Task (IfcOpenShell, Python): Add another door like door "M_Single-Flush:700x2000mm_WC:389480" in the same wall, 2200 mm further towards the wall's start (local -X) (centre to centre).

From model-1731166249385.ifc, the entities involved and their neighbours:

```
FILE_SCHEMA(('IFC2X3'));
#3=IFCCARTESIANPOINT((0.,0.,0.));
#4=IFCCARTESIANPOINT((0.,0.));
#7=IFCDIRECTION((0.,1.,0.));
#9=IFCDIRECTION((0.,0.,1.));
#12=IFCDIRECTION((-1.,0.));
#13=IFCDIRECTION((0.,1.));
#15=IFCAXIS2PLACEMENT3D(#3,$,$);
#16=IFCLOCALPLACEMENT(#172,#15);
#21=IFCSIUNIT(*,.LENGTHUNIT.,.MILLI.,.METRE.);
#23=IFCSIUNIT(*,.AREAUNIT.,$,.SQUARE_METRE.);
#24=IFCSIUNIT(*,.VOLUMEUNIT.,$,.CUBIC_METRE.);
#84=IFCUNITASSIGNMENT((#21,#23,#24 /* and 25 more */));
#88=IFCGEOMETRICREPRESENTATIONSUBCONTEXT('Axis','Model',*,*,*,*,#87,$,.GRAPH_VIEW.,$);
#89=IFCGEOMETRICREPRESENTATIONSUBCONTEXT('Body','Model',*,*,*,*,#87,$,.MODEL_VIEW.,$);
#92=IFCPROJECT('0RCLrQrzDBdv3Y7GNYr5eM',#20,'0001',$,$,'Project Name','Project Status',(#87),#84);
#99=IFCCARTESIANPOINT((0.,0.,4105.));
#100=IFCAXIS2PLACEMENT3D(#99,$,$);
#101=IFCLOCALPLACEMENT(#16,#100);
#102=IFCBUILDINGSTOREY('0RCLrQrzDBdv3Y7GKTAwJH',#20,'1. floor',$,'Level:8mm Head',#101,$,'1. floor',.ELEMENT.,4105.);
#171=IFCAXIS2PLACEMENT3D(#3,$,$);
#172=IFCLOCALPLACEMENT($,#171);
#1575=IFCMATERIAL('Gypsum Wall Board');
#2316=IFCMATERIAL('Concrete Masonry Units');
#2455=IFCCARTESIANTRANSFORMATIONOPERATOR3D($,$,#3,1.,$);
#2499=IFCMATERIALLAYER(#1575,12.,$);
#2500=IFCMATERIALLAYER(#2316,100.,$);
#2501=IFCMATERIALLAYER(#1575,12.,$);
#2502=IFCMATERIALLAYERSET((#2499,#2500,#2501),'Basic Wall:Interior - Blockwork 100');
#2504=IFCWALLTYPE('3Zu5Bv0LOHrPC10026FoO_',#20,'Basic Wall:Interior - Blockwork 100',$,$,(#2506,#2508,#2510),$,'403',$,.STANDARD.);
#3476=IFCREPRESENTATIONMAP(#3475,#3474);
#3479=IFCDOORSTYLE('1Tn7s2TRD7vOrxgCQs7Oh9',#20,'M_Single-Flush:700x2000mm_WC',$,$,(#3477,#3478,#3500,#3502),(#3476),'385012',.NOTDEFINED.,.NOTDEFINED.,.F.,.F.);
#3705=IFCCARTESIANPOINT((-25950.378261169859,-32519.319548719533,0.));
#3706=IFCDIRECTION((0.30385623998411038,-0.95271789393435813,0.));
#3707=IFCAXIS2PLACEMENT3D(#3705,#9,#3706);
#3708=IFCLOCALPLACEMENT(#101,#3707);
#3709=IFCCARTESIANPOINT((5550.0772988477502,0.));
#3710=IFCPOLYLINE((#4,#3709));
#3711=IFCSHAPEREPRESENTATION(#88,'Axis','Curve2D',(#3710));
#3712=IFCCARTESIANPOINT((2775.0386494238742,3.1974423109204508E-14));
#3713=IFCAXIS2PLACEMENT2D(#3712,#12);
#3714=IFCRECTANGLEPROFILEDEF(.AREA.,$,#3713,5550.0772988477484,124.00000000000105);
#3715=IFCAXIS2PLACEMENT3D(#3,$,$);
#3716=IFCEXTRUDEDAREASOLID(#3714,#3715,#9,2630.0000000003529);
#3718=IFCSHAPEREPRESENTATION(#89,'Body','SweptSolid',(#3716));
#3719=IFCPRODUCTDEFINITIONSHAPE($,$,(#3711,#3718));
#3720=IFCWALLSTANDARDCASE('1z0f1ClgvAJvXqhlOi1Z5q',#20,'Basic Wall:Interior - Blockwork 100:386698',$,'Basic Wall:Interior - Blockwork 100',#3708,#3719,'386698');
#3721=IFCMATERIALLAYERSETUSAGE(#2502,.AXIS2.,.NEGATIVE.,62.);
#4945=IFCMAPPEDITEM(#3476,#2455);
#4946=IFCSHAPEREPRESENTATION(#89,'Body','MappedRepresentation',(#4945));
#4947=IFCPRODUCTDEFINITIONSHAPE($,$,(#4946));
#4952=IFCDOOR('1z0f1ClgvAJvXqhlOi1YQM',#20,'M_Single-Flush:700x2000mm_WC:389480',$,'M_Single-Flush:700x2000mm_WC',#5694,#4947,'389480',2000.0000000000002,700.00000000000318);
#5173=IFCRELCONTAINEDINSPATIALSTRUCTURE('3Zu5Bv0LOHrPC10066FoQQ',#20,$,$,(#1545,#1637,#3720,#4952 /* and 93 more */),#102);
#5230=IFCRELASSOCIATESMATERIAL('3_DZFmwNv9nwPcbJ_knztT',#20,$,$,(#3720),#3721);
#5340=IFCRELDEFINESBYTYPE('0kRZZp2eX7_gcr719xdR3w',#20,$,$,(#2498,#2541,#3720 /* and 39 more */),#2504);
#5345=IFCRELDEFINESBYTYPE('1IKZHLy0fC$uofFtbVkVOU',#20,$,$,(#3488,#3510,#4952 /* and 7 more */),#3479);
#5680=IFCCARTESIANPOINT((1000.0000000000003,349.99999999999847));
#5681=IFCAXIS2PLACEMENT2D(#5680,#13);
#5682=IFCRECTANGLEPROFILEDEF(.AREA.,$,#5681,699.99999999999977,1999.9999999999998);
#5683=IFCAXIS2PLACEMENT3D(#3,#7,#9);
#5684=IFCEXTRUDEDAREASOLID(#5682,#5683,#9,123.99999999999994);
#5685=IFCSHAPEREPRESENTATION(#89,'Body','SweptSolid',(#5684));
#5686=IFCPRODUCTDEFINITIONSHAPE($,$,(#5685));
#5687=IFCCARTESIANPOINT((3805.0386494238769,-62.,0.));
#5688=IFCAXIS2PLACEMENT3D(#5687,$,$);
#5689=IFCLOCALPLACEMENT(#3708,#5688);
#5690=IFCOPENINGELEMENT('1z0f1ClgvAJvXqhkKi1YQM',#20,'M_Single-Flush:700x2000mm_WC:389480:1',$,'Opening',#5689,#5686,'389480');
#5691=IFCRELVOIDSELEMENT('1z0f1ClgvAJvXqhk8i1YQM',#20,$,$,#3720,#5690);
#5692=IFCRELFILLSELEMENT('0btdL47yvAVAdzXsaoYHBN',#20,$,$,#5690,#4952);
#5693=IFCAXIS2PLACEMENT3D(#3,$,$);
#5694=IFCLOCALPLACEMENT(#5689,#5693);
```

```python
import ifcopenshell
import ifcopenshell.api.feature
import ifcopenshell.api.geometry
import ifcopenshell.api.root
import ifcopenshell.geom
import ifcopenshell.util.element
import ifcopenshell.util.placement
import ifcopenshell.util.shape

model = ifcopenshell.open("model-1731166249385.ifc")
settings = ifcopenshell.geom.settings()


def volume(element):
    """Net volume in cubic metres, openings subtracted."""
    shape = ifcopenshell.geom.create_shape(settings, element)
    return ifcopenshell.util.shape.get_volume(shape.geometry)


def reuse_history(source, copy):
    """copy_class also copies each property set's owner history, people and application; keep the originals."""
    for rel in copy.IsDefinedBy:
        if rel.is_a("IfcRelDefinesByProperties") and (history := rel.RelatingPropertyDefinition.OwnerHistory):
            rel.RelatingPropertyDefinition.OwnerHistory = source.OwnerHistory
            ifcopenshell.util.element.remove_deep2(model, history)


door = model.by_guid("1z0f1ClgvAJvXqhlOi1YQM")
opening = door.FillsVoids[0].RelatingOpeningElement
wall = opening.VoidsElements[0].RelatingBuildingElement
before = volume(wall)
shift = ifcopenshell.util.placement.get_local_placement(wall.ObjectPlacement)[:3, 0] * -2200.0

# copy_class copies the void relationship, type, container and properties, but no geometry.
new_opening = ifcopenshell.api.root.copy_class(model, product=opening)
new_opening.Representation = ifcopenshell.util.element.copy_deep(
    model, opening.Representation, exclude=["IfcGeometricRepresentationContext", "IfcRepresentationMap"]
)
new_opening.Name = "M_Single-Flush:700x2000mm_WC"
new_opening.Tag = None
new_door = ifcopenshell.api.root.copy_class(model, product=door)
new_door.Representation = ifcopenshell.util.element.copy_deep(
    model, door.Representation, exclude=["IfcGeometricRepresentationContext", "IfcRepresentationMap"]
)
new_door.Name = "M_Single-Flush:700x2000mm_WC"
new_door.Tag = None
reuse_history(door, new_door)
fills = ifcopenshell.api.feature.add_filling(model, opening=new_opening, element=new_door)
fills.OwnerHistory = new_door.OwnerHistory  # required in IFC2X3

for old, new in ((opening, new_opening), (door, new_door)):
    matrix = ifcopenshell.util.placement.get_local_placement(old.ObjectPlacement)
    matrix[:3, 3] += shift
    ifcopenshell.api.geometry.edit_object_placement(model, product=new, matrix=matrix, is_si=False)

after = volume(wall)

print(f"wall volume {before:.3f} -> {after:.3f} m3")

model.write("model-1731166249385_rev.ifc")
```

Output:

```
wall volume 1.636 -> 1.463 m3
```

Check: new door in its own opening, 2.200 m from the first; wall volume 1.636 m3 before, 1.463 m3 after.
